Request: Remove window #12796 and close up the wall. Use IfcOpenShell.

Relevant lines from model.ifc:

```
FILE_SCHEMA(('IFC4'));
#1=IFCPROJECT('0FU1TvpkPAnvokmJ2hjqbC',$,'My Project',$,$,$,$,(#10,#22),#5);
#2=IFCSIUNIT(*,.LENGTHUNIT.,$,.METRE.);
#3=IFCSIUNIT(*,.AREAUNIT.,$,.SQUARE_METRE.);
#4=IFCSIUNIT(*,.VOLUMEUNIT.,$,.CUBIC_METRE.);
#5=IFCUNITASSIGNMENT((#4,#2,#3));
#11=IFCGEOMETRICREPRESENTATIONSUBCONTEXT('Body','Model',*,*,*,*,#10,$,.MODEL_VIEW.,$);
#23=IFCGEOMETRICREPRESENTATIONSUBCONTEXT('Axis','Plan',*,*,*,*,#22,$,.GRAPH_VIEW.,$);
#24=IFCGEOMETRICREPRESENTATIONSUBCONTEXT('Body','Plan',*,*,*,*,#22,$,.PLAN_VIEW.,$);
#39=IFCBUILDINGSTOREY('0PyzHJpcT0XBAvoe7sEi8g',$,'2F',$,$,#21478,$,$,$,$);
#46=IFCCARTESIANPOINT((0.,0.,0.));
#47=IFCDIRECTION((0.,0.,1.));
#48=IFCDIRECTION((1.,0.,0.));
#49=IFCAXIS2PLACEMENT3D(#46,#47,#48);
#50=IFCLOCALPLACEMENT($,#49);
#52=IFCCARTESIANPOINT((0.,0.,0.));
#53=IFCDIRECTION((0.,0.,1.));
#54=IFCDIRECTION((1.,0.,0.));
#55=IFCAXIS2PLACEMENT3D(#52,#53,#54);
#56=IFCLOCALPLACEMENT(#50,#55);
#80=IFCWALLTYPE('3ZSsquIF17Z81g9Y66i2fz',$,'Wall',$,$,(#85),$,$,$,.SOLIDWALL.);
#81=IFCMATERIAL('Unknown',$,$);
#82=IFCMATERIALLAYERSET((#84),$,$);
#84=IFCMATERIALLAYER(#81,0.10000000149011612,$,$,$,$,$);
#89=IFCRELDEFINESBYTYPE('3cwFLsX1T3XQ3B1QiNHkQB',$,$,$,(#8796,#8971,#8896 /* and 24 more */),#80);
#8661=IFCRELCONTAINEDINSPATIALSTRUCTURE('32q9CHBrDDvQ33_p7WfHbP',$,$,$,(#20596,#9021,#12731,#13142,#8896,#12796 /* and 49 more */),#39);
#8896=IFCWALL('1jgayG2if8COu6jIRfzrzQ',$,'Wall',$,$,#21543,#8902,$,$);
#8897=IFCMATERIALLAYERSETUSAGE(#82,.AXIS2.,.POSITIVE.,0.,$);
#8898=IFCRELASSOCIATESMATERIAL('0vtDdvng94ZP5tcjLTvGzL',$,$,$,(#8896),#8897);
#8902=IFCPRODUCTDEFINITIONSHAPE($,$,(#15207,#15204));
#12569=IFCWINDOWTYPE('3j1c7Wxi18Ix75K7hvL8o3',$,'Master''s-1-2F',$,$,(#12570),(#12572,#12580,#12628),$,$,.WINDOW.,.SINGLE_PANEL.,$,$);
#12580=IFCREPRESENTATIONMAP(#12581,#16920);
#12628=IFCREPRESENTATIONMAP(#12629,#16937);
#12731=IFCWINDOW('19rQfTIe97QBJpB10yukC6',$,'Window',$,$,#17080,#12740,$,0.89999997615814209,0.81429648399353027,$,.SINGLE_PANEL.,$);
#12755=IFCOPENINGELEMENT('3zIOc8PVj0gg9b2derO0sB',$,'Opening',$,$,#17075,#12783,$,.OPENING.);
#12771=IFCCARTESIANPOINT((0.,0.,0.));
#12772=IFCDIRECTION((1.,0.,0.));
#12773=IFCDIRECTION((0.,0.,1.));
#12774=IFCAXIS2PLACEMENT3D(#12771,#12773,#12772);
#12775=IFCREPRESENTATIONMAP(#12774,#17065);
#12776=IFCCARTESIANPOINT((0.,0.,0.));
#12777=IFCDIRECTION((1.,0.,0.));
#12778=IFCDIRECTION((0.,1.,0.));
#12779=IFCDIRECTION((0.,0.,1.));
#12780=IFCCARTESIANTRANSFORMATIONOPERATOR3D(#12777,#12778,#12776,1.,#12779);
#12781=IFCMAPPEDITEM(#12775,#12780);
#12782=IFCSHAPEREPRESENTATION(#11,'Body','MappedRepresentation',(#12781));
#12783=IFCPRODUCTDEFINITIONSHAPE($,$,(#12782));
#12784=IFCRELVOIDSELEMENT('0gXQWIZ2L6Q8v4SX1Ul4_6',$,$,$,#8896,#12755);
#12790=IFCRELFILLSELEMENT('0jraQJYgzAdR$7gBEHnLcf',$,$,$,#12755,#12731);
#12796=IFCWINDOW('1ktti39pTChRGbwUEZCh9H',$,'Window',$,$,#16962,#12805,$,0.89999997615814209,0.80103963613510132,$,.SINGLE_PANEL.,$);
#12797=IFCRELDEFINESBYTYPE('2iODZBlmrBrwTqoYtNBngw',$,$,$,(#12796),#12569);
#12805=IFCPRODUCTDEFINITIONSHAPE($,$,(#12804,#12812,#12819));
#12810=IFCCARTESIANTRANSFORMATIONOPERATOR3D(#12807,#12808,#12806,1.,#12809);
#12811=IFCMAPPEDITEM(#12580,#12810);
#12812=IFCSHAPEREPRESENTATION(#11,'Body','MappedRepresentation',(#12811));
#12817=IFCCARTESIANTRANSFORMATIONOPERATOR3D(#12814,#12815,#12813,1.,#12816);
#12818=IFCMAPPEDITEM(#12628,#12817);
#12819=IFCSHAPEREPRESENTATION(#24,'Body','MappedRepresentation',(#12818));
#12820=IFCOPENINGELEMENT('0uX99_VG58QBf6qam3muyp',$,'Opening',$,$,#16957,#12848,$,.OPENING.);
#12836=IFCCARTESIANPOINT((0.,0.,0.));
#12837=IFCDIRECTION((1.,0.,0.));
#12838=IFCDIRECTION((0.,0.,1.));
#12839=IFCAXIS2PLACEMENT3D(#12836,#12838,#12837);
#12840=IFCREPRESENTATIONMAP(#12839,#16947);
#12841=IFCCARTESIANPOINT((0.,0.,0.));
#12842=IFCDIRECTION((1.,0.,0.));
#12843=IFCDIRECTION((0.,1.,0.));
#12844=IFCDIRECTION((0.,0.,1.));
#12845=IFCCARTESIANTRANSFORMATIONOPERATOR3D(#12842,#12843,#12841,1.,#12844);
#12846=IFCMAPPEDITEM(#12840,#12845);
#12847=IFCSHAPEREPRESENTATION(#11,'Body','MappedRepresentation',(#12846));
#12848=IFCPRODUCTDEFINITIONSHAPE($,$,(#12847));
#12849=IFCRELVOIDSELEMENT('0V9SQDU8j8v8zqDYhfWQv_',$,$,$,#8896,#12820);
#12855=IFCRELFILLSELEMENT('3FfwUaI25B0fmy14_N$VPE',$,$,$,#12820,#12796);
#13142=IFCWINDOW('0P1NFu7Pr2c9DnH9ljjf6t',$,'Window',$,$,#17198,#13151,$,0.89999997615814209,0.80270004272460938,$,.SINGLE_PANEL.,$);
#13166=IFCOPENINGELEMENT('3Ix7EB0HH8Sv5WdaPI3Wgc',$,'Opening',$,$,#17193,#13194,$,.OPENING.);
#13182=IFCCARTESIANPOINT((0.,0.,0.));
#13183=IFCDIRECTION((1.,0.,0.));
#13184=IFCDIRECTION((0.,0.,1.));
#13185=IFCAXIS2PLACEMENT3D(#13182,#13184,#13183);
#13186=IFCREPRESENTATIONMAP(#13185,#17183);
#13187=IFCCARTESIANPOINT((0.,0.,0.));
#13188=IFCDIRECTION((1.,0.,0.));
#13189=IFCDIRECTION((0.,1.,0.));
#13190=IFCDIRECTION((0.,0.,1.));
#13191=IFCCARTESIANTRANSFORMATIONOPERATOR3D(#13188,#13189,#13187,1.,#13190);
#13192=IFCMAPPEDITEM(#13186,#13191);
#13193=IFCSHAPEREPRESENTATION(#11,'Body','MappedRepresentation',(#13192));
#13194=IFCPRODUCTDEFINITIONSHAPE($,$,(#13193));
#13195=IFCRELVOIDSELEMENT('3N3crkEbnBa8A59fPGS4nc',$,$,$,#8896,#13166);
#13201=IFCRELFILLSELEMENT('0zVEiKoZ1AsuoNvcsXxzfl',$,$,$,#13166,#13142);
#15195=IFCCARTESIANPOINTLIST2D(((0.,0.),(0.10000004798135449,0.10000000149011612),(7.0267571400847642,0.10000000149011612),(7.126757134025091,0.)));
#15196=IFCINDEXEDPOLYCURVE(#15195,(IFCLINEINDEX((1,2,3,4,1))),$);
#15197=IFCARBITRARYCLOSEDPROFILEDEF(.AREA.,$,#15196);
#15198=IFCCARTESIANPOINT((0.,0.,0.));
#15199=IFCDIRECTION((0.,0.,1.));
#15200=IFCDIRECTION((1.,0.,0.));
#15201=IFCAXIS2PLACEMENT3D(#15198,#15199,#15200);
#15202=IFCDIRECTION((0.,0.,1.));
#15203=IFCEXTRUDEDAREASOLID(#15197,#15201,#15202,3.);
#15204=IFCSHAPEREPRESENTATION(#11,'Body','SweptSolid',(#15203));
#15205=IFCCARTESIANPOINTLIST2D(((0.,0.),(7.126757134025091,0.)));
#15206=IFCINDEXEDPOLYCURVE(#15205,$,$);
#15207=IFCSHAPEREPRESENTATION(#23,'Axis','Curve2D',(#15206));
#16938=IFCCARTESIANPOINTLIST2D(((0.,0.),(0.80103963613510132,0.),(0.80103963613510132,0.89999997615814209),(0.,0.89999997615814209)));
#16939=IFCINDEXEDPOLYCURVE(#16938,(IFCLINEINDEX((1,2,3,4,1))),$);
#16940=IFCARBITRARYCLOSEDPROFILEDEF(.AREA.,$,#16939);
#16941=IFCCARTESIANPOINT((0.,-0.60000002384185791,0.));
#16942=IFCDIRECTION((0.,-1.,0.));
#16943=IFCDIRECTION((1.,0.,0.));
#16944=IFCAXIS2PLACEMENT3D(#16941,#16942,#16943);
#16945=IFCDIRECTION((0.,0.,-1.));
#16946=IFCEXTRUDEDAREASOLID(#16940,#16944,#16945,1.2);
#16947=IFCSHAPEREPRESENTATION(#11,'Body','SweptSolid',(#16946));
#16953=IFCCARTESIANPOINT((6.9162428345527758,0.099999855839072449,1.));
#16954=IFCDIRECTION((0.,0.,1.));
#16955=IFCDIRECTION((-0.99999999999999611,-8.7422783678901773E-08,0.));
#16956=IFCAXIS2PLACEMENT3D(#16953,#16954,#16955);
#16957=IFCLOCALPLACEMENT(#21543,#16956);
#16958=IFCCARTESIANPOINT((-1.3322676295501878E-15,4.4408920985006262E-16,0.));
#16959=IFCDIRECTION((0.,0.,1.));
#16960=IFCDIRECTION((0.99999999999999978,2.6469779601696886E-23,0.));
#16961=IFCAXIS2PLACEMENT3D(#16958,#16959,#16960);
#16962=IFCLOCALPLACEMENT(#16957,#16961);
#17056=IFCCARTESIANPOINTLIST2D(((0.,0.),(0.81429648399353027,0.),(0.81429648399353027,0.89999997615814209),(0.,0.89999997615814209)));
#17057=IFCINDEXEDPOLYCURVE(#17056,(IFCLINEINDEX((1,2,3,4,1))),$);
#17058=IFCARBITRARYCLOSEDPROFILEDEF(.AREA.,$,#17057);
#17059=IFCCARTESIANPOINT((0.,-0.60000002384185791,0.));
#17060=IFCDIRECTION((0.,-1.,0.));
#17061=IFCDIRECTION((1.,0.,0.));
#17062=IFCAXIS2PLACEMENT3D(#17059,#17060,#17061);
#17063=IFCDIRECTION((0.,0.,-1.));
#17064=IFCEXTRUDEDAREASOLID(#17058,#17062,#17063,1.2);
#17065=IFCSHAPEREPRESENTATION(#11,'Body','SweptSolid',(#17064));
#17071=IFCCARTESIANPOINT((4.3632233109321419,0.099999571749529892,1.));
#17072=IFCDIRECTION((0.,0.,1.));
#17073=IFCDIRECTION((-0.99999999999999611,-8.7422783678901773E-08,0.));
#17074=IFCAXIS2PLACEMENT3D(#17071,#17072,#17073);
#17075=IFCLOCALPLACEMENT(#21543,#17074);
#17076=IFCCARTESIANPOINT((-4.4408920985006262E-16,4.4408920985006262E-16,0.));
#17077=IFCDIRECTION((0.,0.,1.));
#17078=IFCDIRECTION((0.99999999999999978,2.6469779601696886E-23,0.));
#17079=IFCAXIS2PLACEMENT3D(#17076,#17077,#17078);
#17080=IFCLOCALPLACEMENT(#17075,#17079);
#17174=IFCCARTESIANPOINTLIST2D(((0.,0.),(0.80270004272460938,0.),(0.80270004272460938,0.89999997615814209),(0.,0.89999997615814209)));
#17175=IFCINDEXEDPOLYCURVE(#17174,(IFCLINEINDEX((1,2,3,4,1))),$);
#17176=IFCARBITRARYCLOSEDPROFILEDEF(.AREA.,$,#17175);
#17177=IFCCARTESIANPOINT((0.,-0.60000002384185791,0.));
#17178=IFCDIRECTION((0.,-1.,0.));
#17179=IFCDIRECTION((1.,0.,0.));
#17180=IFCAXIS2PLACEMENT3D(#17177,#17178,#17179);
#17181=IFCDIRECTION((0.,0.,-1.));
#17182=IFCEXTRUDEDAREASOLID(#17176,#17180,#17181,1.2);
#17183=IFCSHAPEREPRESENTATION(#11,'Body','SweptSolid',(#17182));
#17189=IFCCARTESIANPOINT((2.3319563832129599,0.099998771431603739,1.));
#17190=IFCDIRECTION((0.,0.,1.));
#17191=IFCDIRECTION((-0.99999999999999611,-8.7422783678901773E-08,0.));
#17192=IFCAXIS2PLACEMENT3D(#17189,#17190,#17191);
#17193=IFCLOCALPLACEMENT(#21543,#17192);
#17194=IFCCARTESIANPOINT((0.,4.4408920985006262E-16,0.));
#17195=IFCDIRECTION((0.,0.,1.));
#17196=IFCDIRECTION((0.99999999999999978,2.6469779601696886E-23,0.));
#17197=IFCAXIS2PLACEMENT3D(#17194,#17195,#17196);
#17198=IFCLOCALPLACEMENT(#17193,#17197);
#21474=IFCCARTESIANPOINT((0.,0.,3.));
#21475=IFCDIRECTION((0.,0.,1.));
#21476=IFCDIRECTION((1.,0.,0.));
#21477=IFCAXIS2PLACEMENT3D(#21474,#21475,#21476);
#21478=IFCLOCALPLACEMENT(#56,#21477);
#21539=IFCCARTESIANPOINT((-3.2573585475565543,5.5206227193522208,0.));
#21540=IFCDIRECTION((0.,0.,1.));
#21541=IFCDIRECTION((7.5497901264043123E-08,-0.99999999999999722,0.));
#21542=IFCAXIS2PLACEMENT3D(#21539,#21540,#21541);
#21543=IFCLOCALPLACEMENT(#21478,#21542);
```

```python
import ifcopenshell
import ifcopenshell.api.feature
import ifcopenshell.api.root
import ifcopenshell.geom
import ifcopenshell.util.shape

model = ifcopenshell.open("model.ifc")
settings = ifcopenshell.geom.settings()


def volume(element):
    """Net volume in cubic metres, openings subtracted."""
    shape = ifcopenshell.geom.create_shape(settings, element)
    return ifcopenshell.util.shape.get_volume(shape.geometry)


window = model.by_guid("1ktti39pTChRGbwUEZCh9H")
opening = window.FillsVoids[0].RelatingOpeningElement
wall = opening.VoidsElements[0].RelatingBuildingElement
before = volume(wall)

ifcopenshell.api.root.remove_product(model, product=window)
ifcopenshell.api.feature.remove_feature(model, feature=opening)

after = volume(wall)

print(f"wall volume {before:.3f} -> {after:.3f} m3")

model.write("model_v2.ifc")
```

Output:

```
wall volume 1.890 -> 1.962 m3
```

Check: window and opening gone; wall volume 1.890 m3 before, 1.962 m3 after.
